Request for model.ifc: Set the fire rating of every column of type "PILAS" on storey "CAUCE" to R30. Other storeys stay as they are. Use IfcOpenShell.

First a look at what the model holds.

```python
import ifcopenshell
import ifcopenshell.util.element

model = ifcopenshell.open("model.ifc")
print(model.schema)
storey = next(s for s in model.by_type("IfcBuildingStorey") if s.Name == "CAUCE")
columns = [e for e in ifcopenshell.util.element.get_decomposition(storey) if e.is_a("IfcColumn")]
seen = {}
for e in columns:
    element_type = ifcopenshell.util.element.get_type(e)
    key = (element_type.Name if element_type != e and element_type else None, ifcopenshell.util.element.get_pset(e, "Pset_ColumnCommon", "FireRating"))
    seen[key] = seen.get(key, 0) + 1
for (name, value), count in sorted(seen.items(), key=str):
    print(count, "x", name, "|", value)
```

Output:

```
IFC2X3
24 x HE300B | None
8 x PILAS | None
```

```python
import ifcopenshell
import ifcopenshell.api.pset
import ifcopenshell.util.element

model = ifcopenshell.open("model.ifc")

storey = next(s for s in model.by_type("IfcBuildingStorey") if s.Name == "CAUCE")
columns = [e for e in ifcopenshell.util.element.get_decomposition(storey) if e.is_a("IfcColumn")]

count = 0
for e in columns:
    element_type = ifcopenshell.util.element.get_type(e)
    if element_type in (None, e) or element_type.Name != "PILAS":
        continue
    # add_pset returns the element's existing set when there is one.
    pset = ifcopenshell.api.pset.add_pset(model, product=e, name="Pset_ColumnCommon")
    ifcopenshell.api.pset.edit_pset(model, pset=pset, properties={"FireRating": "R30"})
    count += 1

print(count, "columns updated")

model.write("model_rev.ifc")
```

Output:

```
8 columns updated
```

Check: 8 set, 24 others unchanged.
